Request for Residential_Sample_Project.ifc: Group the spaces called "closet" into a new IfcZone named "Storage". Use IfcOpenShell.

First a look at what the model holds.

```python
import ifcopenshell

model = ifcopenshell.open("Residential_Sample_Project.ifc")
print(model.schema)
seen = {}
for space in model.by_type("IfcSpace"):
    seen[space.LongName] = seen.get(space.LongName, 0) + 1
for name, count in sorted(seen.items(), key=str):
    print(count, "x", name)
print("zones:", [z.Name for z in model.by_type("IfcZone")][:20])
```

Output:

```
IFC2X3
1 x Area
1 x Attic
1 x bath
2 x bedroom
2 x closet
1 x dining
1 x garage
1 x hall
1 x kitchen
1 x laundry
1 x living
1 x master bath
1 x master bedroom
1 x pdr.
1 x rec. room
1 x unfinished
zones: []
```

```python
import ifcopenshell
import ifcopenshell.api.group
import ifcopenshell.api.root

model = ifcopenshell.open("Residential_Sample_Project.ifc")

names = {"closet"}
spaces = [s for s in model.by_type("IfcSpace") if s.LongName in names]

zone = ifcopenshell.api.root.create_entity(model, ifc_class="IfcZone", name="Storage")
ifcopenshell.api.group.assign_group(model, products=spaces, group=zone)
print(len(spaces), "spaces in", zone.Name)

model.write("Residential_Sample_Project_rev.ifc")
```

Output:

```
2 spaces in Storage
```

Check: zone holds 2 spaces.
